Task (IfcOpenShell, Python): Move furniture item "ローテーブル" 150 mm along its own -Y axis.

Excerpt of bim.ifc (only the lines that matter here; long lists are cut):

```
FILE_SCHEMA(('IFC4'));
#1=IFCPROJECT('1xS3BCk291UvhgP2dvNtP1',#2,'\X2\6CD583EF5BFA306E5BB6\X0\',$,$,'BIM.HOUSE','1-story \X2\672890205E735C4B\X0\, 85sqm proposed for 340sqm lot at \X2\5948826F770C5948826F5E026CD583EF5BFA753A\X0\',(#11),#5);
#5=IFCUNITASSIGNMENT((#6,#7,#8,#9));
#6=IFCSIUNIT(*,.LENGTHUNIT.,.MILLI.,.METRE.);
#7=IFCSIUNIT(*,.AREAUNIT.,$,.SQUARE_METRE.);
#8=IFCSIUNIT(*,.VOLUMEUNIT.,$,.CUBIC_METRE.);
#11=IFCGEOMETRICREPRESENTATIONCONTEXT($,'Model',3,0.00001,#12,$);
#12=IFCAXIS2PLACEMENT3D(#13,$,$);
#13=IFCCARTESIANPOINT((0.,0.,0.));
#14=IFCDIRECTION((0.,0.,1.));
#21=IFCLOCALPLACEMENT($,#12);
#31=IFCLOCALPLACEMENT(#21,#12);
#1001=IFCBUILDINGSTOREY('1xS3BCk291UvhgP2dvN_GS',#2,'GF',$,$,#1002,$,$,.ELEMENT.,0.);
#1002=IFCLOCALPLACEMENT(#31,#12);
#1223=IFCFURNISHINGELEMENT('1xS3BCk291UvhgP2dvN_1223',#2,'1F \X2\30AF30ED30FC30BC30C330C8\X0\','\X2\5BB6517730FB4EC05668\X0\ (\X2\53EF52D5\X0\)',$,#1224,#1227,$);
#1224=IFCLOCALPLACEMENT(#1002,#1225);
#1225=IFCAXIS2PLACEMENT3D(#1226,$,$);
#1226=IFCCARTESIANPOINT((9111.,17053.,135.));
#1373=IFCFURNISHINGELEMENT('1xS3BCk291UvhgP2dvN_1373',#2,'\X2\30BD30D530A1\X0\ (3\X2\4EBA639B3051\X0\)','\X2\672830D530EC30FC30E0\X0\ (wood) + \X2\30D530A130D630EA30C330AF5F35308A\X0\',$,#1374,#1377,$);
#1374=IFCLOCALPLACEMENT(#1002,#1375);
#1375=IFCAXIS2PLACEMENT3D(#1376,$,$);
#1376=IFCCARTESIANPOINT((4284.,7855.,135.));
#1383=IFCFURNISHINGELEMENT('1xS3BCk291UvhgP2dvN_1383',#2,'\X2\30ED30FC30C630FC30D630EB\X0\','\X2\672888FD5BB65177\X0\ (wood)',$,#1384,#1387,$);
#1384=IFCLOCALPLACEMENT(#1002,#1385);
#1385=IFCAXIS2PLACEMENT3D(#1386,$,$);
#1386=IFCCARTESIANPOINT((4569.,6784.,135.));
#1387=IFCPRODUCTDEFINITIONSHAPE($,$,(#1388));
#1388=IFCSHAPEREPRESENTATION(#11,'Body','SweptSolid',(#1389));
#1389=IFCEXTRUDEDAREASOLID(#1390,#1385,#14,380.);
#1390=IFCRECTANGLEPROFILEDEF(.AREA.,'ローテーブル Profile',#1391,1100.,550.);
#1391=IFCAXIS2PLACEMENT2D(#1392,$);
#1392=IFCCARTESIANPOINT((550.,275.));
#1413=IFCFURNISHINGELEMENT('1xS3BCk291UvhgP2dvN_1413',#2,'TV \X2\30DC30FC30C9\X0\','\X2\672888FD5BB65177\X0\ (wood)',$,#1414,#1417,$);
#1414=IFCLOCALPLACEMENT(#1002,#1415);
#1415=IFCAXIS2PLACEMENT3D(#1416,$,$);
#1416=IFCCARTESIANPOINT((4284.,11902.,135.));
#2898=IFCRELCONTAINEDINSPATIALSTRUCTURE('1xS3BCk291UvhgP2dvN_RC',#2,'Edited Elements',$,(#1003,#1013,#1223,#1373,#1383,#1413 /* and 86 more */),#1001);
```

```python
import ifcopenshell
import ifcopenshell.api.geometry
import ifcopenshell.util.placement
import ifcopenshell.util.unit

model = ifcopenshell.open("bim.ifc")
unit_scale = ifcopenshell.util.unit.calculate_unit_scale(model)

item = model.by_id(1383)
matrix = ifcopenshell.util.placement.get_local_placement(item.ObjectPlacement)
matrix[:3, 3] -= matrix[:3, 1] * 0.15 / unit_scale
ifcopenshell.api.geometry.edit_object_placement(model, product=item, matrix=matrix, is_si=False)

print(ifcopenshell.util.placement.get_local_placement(item.ObjectPlacement).round(3) + 0.0)

model.write("bim_v2.ifc")
```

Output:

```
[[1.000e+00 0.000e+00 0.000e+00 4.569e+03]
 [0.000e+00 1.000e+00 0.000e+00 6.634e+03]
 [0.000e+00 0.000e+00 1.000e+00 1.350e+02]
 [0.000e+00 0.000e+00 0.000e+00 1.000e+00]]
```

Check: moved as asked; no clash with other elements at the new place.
